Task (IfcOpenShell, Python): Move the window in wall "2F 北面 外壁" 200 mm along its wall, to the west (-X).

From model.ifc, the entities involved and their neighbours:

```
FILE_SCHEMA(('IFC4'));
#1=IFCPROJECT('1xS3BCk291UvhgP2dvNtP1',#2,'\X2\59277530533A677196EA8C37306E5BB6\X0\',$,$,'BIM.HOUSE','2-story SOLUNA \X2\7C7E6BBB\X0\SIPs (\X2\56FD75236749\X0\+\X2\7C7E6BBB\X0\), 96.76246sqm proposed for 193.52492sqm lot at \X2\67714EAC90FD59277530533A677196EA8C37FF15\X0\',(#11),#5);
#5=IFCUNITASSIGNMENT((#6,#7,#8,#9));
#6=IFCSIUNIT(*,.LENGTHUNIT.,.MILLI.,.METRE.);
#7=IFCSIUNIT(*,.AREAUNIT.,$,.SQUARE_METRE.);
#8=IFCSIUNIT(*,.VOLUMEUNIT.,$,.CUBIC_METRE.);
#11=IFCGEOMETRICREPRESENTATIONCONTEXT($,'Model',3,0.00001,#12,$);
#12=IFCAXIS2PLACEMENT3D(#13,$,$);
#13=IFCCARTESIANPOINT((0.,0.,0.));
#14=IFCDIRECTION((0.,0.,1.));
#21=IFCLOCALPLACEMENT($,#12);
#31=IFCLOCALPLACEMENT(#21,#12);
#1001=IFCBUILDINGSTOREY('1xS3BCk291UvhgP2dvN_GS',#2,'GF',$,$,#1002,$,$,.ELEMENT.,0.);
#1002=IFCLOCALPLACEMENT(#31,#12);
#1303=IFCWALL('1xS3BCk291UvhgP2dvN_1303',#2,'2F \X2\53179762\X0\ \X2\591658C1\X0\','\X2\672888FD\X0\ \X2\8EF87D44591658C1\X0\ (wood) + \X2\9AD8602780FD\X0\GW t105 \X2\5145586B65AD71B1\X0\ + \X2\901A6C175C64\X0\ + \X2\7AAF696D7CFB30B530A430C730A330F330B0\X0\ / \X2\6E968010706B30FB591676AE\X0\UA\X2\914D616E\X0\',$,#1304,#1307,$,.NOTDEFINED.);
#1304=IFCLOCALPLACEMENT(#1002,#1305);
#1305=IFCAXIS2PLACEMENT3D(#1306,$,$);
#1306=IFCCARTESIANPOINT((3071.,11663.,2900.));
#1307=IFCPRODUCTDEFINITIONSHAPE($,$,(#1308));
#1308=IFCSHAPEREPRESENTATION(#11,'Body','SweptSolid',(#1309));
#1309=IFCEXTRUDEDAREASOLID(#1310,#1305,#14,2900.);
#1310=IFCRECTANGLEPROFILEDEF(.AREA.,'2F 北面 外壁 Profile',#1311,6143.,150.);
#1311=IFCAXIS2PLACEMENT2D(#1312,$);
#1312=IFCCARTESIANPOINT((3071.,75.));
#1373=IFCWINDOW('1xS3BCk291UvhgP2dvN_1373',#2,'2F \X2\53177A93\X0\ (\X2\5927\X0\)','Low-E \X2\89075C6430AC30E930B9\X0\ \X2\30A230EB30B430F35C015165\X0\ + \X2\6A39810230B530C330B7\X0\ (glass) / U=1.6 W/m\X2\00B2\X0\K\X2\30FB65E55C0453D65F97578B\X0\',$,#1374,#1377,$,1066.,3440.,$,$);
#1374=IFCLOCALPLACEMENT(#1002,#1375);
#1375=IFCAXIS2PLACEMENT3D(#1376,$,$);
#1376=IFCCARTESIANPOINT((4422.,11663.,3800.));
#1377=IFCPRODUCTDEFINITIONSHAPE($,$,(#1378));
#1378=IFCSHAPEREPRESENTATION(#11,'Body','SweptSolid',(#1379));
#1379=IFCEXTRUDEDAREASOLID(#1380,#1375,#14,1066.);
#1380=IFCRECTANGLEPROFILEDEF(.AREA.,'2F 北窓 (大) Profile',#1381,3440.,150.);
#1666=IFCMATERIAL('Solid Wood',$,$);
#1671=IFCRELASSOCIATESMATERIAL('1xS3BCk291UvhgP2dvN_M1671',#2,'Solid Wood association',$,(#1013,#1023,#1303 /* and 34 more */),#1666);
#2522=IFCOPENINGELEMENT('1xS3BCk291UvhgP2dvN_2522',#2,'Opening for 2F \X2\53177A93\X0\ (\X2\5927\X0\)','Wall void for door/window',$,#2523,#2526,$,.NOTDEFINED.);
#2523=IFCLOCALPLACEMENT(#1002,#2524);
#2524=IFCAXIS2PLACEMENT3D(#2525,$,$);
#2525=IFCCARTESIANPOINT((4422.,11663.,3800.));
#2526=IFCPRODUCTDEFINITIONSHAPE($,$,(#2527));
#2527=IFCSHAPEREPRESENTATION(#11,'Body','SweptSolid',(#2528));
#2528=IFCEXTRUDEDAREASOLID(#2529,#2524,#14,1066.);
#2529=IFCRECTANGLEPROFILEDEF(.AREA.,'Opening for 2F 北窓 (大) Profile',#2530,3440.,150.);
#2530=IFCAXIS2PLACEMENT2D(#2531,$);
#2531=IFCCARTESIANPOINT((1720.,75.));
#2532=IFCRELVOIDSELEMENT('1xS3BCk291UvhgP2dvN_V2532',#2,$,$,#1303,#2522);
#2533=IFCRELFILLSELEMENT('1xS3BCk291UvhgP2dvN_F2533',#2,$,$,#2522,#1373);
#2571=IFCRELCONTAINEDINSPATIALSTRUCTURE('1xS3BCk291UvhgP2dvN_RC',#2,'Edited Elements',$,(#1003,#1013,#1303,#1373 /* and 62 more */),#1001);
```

```python
import ifcopenshell
import ifcopenshell.api.geometry
import ifcopenshell.util.placement
import ifcopenshell.util.unit

model = ifcopenshell.open("model.ifc")
unit_scale = ifcopenshell.util.unit.calculate_unit_scale(model)

window = model.by_guid("1xS3BCk291UvhgP2dvN_1373")
opening = window.FillsVoids[0].RelatingOpeningElement
wall = opening.VoidsElements[0].RelatingBuildingElement

wall_matrix = ifcopenshell.util.placement.get_local_placement(wall.ObjectPlacement)
shift = wall_matrix[:3, 0] * -0.2 / unit_scale
before = ifcopenshell.util.placement.get_local_placement(window.ObjectPlacement)[:3, 3].copy()

# The window is not placed relative to its opening, so move both.
for product in (opening, window):
    matrix = ifcopenshell.util.placement.get_local_placement(product.ObjectPlacement)
    matrix[:3, 3] += shift
    ifcopenshell.api.geometry.edit_object_placement(model, product=product, matrix=matrix, is_si=False)

after = ifcopenshell.util.placement.get_local_placement(window.ObjectPlacement)[:3, 3]
print("window moved by", (after - before).round(3) + 0.0)

model.write("model_updated.ifc")
```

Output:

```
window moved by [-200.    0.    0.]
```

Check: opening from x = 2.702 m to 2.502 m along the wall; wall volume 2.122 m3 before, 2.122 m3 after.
